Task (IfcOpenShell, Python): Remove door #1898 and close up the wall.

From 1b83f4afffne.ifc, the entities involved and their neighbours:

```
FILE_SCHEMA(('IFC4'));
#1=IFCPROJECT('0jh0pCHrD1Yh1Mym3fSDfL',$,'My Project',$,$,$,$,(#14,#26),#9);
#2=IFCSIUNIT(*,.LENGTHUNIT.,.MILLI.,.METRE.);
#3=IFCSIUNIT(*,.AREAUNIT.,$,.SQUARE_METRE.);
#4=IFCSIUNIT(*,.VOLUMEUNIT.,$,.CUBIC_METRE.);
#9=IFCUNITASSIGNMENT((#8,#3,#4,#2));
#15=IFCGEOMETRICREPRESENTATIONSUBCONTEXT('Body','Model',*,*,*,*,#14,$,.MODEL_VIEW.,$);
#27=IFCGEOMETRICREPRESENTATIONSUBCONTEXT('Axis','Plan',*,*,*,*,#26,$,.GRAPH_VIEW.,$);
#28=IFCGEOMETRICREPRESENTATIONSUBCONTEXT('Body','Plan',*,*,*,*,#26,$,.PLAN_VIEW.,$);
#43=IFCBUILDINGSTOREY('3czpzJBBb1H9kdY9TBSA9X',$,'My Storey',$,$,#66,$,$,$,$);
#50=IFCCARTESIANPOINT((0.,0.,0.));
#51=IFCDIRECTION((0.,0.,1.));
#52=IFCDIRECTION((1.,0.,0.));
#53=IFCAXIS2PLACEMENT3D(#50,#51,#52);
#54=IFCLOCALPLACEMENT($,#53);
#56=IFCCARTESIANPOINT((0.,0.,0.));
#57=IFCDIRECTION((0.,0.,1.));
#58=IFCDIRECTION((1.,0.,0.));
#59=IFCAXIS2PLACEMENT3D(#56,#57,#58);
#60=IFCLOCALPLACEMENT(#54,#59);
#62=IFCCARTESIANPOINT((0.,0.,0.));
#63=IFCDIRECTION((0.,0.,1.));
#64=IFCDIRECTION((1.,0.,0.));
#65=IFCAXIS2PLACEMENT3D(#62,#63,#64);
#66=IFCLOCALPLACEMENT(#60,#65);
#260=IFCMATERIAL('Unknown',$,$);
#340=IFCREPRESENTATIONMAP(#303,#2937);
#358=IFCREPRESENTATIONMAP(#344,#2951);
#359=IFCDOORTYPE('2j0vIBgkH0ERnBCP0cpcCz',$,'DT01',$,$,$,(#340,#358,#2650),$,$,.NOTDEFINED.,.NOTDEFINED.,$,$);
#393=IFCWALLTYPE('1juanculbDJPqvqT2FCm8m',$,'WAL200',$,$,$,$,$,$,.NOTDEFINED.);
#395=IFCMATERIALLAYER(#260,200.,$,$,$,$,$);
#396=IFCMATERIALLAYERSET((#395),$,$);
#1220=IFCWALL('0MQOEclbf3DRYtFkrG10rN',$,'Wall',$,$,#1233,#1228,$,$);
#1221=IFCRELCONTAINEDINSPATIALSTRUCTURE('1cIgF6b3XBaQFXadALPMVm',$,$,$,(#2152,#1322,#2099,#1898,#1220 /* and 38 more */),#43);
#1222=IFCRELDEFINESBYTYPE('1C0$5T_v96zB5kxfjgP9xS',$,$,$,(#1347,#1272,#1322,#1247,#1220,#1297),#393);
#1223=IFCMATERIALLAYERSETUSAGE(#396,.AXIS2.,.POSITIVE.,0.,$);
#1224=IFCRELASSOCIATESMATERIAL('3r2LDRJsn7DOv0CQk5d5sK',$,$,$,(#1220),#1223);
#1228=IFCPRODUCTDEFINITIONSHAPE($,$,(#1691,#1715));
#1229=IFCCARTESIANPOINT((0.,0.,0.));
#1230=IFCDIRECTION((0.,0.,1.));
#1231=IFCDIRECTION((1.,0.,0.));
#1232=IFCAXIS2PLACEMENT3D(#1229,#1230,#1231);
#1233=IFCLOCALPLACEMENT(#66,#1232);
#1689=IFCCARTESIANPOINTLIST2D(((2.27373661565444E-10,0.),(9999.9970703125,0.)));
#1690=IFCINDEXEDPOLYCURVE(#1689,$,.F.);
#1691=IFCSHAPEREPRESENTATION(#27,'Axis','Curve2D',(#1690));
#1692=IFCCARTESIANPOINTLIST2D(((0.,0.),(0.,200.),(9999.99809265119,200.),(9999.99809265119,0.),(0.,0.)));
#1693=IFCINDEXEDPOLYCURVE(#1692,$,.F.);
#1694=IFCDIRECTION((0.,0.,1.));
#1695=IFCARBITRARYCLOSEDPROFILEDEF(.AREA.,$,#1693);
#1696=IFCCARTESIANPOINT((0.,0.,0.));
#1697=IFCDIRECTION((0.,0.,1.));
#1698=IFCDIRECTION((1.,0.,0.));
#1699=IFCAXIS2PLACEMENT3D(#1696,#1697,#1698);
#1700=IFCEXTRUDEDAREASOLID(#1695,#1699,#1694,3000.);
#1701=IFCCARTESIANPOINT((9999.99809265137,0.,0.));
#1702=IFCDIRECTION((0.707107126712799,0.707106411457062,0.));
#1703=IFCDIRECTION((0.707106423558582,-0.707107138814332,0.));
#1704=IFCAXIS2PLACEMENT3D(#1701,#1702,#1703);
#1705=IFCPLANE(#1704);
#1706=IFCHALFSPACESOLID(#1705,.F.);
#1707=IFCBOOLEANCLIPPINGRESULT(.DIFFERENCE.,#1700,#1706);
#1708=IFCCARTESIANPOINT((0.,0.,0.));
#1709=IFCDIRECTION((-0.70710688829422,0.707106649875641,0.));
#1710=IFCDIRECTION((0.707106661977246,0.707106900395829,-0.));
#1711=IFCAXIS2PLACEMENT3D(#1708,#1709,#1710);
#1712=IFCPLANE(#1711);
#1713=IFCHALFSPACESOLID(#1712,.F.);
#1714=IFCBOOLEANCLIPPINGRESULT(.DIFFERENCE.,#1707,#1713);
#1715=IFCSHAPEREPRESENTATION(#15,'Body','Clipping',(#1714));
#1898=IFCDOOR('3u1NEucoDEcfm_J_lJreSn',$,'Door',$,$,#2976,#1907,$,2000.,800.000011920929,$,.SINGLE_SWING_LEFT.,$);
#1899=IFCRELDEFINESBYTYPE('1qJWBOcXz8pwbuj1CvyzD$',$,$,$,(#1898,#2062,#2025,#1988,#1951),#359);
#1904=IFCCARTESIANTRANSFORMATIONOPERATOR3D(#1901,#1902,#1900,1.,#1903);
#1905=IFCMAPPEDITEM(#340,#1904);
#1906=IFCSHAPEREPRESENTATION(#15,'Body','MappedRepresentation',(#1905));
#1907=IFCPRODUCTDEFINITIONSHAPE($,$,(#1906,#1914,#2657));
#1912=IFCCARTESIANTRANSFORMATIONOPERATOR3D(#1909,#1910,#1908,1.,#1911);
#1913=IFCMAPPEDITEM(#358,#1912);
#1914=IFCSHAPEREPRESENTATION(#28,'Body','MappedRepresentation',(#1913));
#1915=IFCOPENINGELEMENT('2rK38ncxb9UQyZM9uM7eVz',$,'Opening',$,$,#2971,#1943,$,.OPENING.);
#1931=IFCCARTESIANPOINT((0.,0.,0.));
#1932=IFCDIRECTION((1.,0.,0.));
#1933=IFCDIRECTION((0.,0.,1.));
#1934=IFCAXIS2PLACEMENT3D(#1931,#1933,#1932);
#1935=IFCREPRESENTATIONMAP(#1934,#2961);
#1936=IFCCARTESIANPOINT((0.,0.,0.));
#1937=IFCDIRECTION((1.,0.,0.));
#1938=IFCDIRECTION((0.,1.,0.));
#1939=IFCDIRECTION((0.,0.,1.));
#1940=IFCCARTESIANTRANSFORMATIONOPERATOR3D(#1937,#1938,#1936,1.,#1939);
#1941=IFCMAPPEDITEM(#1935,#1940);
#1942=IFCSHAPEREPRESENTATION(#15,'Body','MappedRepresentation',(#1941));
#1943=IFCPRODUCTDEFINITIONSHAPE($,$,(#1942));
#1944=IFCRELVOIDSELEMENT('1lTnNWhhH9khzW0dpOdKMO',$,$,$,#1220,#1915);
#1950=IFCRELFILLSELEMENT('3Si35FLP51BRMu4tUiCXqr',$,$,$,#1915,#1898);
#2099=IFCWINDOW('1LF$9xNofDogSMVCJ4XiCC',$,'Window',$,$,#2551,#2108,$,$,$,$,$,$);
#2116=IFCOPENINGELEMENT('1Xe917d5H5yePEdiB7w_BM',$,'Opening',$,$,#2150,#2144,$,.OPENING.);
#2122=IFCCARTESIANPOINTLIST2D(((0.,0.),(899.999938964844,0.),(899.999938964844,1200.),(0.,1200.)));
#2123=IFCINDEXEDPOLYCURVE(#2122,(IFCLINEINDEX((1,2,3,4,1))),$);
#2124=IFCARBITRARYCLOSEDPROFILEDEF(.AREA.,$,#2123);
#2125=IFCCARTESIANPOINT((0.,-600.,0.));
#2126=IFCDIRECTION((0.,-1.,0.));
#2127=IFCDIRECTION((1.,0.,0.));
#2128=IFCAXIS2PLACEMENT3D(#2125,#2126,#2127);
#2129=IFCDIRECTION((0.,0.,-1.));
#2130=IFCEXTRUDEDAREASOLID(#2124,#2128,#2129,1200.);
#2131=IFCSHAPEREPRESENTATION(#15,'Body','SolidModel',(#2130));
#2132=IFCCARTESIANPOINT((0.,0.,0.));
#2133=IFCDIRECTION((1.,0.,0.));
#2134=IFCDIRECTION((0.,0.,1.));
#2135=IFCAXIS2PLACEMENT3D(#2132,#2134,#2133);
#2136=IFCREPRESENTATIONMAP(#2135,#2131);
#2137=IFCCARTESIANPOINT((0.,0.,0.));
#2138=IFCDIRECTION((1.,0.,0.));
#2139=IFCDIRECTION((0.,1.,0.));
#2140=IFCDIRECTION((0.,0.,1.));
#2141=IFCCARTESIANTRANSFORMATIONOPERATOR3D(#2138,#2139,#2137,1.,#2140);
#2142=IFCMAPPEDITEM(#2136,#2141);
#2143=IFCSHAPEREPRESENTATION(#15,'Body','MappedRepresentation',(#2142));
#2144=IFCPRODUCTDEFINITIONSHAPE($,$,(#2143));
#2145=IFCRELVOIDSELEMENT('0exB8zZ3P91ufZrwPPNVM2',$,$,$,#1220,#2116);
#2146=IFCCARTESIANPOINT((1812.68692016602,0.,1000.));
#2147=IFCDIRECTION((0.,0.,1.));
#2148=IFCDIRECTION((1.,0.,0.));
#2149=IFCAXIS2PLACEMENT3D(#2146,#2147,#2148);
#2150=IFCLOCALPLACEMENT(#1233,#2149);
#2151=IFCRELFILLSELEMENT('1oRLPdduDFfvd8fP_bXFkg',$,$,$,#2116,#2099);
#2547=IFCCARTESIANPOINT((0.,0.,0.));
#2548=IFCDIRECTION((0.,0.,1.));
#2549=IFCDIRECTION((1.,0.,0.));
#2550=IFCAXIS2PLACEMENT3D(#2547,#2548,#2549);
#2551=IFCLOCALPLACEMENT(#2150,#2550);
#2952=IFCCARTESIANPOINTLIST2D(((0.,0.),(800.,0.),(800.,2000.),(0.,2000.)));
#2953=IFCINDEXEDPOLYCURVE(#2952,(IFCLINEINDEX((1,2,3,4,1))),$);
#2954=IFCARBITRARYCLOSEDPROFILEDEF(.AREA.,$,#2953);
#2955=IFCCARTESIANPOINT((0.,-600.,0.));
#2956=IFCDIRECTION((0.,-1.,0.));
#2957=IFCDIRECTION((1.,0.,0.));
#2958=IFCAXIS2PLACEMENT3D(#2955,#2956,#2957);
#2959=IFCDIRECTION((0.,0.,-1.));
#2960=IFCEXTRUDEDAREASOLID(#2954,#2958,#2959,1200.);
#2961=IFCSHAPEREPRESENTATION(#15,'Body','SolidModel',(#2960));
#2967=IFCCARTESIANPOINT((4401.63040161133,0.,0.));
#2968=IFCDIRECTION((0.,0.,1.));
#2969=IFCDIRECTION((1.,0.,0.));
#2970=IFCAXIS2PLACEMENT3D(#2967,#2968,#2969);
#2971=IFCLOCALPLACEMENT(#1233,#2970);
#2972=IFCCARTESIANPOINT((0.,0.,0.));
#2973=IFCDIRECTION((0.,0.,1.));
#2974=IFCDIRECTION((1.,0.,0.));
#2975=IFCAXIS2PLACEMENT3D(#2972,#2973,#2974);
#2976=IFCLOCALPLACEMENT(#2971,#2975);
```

```python
import ifcopenshell
import ifcopenshell.api.feature
import ifcopenshell.api.root
import ifcopenshell.geom
import ifcopenshell.util.shape

model = ifcopenshell.open("1b83f4afffne.ifc")
settings = ifcopenshell.geom.settings()


def volume(element):
    """Net volume in cubic metres, openings subtracted."""
    shape = ifcopenshell.geom.create_shape(settings, element)
    return ifcopenshell.util.shape.get_volume(shape.geometry)


door = model.by_guid("3u1NEucoDEcfm_J_lJreSn")
opening = door.FillsVoids[0].RelatingOpeningElement
wall = opening.VoidsElements[0].RelatingBuildingElement
before = volume(wall)

ifcopenshell.api.root.remove_product(model, product=door)
ifcopenshell.api.feature.remove_feature(model, feature=opening)

after = volume(wall)

print(f"wall volume {before:.3f} -> {after:.3f} m3")

model.write("1b83f4afffne_rev.ifc")
```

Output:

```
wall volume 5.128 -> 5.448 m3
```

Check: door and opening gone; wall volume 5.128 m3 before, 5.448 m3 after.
